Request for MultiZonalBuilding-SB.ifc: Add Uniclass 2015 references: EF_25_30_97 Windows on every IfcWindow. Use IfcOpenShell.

First a look at what the model holds.

```python
import ifcopenshell

model = ifcopenshell.open("MultiZonalBuilding-SB.ifc")
print(model.schema)
print("classifications:", [c.Name for c in model.by_type("IfcClassification")])
for ifc_class in ("IfcDoor", "IfcRoof", "IfcStair", "IfcWall", "IfcWindow"):
    print(ifc_class, len(model.by_type(ifc_class)))
```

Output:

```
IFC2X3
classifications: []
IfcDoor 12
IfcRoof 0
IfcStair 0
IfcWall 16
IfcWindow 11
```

```python
import ifcopenshell
import ifcopenshell.api.classification

model = ifcopenshell.open("MultiZonalBuilding-SB.ifc")

# IFC2X3 requires Source and Edition and has no link from the project to the system.
system = model.create_entity("IfcClassification", Source="NBS", Edition="2015", Name="Uniclass 2015")

codes = {
    "IfcWindow": ("EF_25_30_97", "Windows"),
}
for ifc_class, (code, name) in codes.items():
    products = model.by_type(ifc_class)
    ifcopenshell.api.classification.add_reference(
        model, products=products, classification=system, identification=code, name=name
    )
    print(code, len(products))

model.write("MultiZonalBuilding-SB_rev.ifc")
```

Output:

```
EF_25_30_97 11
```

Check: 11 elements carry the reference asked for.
